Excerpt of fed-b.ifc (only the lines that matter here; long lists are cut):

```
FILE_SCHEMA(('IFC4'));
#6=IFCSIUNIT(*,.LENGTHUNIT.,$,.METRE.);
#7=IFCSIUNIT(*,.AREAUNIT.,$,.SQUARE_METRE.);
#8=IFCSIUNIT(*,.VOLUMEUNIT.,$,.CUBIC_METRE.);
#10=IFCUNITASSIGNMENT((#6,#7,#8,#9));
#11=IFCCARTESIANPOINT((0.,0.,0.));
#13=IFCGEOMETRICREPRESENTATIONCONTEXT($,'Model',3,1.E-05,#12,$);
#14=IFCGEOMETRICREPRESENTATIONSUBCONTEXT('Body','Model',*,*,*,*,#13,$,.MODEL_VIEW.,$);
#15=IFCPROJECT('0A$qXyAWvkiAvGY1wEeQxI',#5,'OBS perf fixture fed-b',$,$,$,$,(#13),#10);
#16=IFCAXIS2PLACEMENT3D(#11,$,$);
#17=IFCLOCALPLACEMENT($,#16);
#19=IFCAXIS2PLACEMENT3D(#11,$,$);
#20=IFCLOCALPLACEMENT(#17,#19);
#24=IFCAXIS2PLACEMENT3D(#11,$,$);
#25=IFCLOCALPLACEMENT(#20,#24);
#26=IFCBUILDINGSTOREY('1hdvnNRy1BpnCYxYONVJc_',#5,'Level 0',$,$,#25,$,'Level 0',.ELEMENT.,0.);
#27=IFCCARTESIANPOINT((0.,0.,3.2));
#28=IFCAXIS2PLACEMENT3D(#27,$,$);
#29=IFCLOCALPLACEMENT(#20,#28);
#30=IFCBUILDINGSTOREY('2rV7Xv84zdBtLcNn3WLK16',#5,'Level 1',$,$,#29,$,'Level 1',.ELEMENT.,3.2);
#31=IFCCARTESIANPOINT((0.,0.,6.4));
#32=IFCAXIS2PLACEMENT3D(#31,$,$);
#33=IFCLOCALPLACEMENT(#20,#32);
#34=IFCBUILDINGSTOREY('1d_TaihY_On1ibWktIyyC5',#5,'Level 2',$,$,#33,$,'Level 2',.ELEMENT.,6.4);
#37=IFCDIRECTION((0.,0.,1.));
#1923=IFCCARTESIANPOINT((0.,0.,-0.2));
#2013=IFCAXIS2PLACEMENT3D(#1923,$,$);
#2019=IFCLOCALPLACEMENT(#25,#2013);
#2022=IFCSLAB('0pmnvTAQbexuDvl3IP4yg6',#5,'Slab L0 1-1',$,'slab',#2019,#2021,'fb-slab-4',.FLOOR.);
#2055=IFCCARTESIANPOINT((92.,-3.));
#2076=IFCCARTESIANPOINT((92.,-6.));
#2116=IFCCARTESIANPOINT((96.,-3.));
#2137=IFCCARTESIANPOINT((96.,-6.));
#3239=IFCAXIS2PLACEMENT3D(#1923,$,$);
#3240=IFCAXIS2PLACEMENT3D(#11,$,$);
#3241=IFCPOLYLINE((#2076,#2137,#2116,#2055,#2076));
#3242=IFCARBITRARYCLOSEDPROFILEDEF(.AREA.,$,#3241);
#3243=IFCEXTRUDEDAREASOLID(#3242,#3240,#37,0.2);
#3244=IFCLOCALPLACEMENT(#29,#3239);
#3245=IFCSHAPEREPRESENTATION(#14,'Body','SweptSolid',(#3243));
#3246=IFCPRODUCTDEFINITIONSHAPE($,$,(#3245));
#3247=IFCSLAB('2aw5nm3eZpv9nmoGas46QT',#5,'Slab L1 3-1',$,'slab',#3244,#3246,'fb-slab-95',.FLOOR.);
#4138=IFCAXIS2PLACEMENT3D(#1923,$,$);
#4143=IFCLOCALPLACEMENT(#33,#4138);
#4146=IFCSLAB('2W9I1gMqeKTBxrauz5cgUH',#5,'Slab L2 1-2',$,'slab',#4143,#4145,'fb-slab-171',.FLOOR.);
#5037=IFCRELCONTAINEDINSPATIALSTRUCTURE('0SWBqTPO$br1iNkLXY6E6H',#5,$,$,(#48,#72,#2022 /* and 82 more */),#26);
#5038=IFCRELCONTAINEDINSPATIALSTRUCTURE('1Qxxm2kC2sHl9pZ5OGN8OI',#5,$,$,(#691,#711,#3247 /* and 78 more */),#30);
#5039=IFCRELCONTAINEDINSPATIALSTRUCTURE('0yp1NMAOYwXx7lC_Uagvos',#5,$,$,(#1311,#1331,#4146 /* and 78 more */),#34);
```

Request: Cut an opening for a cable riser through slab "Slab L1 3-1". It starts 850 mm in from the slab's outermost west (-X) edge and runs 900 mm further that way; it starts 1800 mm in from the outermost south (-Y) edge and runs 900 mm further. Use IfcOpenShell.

```python
import numpy as np
import ifcopenshell
import ifcopenshell.api.feature
import ifcopenshell.api.geometry
import ifcopenshell.api.root
import ifcopenshell.geom
import ifcopenshell.util.placement
import ifcopenshell.util.representation
import ifcopenshell.util.shape
import ifcopenshell.util.unit

model = ifcopenshell.open("fed-b.ifc")
unit_scale = ifcopenshell.util.unit.calculate_unit_scale(model)
settings = ifcopenshell.geom.settings()


def volume(element):
    """Net volume in cubic metres, openings subtracted."""
    shape = ifcopenshell.geom.create_shape(settings, element)
    return ifcopenshell.util.shape.get_volume(shape.geometry)


slab = model.by_guid("2aw5nm3eZpv9nmoGas46QT")
before = volume(slab)

# Extent in the slab's own axes, in metres. The edges named are its -X and -Y sides.
slab_shape = ifcopenshell.geom.create_shape(settings, slab)
vertices = ifcopenshell.util.shape.get_vertices(slab_shape.geometry)
x_min, y_min, bottom = vertices.min(axis=0)
top = vertices[:, 2].max()

opening = ifcopenshell.api.root.create_entity(model, ifc_class="IfcOpeningElement", name="Cable riser opening", predefined_type="OPENING")
context = ifcopenshell.util.representation.get_context(model, "Model", "Body", "MODEL_VIEW")
width, depth = 0.9, 0.9
outline = [(0.0, 0.0), (width, 0.0), (width, depth), (0.0, depth), (0.0, 0.0)]
# Overshoot both faces by 50 mm so the cut is clean.
shape = ifcopenshell.api.geometry.add_slab_representation(
    model, context=context, depth=top - bottom + 0.1, polyline=outline
)
ifcopenshell.api.geometry.assign_representation(model, product=opening, representation=shape)

matrix = ifcopenshell.util.placement.get_local_placement(slab.ObjectPlacement)
matrix[:, 3] = matrix @ np.append(np.array([x_min + 0.85, y_min + 1.8, bottom - 0.05]) / unit_scale, 1.0)
ifcopenshell.api.geometry.edit_object_placement(model, product=opening, matrix=matrix, is_si=False)
ifcopenshell.api.feature.add_feature(model, feature=opening, element=slab)

after = volume(slab)

print(f"slab volume {before:.3f} -> {after:.3f} m3")

model.write("fed-b_updated.ifc")
```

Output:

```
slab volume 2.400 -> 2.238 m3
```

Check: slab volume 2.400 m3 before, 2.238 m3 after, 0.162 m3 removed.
